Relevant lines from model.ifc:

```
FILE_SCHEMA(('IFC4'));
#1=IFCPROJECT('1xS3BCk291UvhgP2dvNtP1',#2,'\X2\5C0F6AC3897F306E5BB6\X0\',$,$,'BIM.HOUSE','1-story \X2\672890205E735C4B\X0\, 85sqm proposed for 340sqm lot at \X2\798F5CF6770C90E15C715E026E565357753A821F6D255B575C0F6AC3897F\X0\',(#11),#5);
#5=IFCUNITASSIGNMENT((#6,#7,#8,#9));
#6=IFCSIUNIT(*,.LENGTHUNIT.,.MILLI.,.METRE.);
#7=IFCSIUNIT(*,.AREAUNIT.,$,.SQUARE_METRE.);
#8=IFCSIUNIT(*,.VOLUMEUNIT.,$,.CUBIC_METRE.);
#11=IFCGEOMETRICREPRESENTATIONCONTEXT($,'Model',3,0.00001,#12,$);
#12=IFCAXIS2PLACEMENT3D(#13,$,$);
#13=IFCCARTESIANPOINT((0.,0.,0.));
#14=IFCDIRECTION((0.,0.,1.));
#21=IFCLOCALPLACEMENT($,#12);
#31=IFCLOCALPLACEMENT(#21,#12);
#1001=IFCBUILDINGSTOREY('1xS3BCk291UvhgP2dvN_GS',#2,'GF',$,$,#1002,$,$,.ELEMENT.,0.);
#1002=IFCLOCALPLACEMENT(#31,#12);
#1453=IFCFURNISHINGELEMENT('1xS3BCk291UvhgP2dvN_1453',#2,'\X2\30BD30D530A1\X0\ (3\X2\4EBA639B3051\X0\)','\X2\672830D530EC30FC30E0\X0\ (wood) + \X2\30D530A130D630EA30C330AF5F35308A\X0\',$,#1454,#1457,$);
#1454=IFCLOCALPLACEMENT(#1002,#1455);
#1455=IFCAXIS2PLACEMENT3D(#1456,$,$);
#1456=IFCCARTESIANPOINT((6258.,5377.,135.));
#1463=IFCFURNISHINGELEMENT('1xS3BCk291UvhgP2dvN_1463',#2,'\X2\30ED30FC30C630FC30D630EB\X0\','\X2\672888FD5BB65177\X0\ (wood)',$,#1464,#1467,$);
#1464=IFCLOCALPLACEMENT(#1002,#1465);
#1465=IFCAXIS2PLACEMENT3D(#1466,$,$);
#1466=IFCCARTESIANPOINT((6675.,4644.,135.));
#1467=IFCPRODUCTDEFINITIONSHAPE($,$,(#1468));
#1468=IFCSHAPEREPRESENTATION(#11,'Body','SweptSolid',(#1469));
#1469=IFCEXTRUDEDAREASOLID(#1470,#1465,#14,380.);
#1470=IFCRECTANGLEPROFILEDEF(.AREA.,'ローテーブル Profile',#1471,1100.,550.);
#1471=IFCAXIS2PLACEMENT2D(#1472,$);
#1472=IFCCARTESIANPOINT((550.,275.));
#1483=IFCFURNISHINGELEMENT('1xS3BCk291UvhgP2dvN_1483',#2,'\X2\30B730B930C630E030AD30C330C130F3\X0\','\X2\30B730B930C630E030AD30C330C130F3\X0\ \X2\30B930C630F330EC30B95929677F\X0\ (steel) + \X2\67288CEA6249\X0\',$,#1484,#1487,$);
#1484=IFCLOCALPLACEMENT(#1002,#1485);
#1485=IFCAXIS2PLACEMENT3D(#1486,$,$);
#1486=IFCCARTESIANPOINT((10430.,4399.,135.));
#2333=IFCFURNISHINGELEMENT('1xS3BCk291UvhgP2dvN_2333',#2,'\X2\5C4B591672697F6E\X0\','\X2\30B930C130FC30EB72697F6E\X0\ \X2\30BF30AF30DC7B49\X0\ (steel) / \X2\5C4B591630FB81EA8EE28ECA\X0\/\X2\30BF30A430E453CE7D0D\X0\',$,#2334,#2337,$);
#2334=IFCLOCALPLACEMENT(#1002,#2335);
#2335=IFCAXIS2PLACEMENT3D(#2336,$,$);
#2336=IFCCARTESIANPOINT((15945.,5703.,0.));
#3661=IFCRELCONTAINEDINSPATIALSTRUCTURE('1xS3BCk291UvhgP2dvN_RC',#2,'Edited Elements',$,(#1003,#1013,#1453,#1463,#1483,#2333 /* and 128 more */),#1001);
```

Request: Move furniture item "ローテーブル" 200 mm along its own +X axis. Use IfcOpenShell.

```python
import ifcopenshell
import ifcopenshell.api.geometry
import ifcopenshell.util.placement

model = ifcopenshell.open("model.ifc")

item = model.by_guid("1xS3BCk291UvhgP2dvN_1463")
matrix = ifcopenshell.util.placement.get_local_placement(item.ObjectPlacement)
matrix[:3, 3] += matrix[:3, 0] * 200.0
ifcopenshell.api.geometry.edit_object_placement(model, product=item, matrix=matrix, is_si=False)

print(ifcopenshell.util.placement.get_local_placement(item.ObjectPlacement).round(3) + 0.0)

model.write("model_updated.ifc")
```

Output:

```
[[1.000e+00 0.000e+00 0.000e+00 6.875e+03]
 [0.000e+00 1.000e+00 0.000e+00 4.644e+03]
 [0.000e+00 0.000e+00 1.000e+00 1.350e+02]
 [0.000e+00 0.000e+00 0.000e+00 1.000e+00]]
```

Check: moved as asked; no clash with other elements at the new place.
